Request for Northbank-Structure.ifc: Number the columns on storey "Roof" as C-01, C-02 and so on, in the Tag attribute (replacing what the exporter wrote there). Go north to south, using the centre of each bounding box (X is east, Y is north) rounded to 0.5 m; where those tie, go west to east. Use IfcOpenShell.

First a look at what the model holds.

```python
import ifcopenshell
import ifcopenshell.util.element
import ifcopenshell.util.placement

model = ifcopenshell.open("Northbank-Structure.ifc")
print(model.schema)
storey = next(s for s in model.by_type("IfcBuildingStorey") if s.Name == "Roof")
columns = [e for e in ifcopenshell.util.element.get_decomposition(storey) if e.is_a("IfcColumn")]
for e in sorted(columns, key=lambda e: e.id()):
    origin = ifcopenshell.util.placement.get_local_placement(e.ObjectPlacement)[:3, 3]
    print(e.id(), e.Tag, e.Name, origin.round(2) + 0.0, sep=" | ")
```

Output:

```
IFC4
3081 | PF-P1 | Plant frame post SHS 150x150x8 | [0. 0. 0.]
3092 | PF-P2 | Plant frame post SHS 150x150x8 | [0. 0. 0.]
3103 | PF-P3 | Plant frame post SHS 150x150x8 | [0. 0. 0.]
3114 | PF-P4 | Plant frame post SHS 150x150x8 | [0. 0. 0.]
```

```python
import ifcopenshell
import ifcopenshell.geom
import ifcopenshell.util.element
import ifcopenshell.util.shape

model = ifcopenshell.open("Northbank-Structure.ifc")
settings = ifcopenshell.geom.settings()
settings.set("use-world-coords", True)


def centre(element):
    shape = ifcopenshell.geom.create_shape(settings, element)
    return ifcopenshell.util.shape.get_bbox_centroid(shape.geometry)


storey = next(s for s in model.by_type("IfcBuildingStorey") if s.Name == "Roof")
columns = [e for e in ifcopenshell.util.element.get_decomposition(storey) if e.is_a("IfcColumn")]

# Insertion points can sit at a corner or the storey origin, so sort by the geometry (in metres).
centres = {e: centre(e) for e in columns}
columns.sort(key=lambda e: (-round(centres[e][1] / 0.5), centres[e][0]))

for i, e in enumerate(columns, start=1):
    number = f"C-{i:02d}"
    e.Tag = number
    print(e.id(), number)

model.write("Northbank-Structure_rev.ifc")
```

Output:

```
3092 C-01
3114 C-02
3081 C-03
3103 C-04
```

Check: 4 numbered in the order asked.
